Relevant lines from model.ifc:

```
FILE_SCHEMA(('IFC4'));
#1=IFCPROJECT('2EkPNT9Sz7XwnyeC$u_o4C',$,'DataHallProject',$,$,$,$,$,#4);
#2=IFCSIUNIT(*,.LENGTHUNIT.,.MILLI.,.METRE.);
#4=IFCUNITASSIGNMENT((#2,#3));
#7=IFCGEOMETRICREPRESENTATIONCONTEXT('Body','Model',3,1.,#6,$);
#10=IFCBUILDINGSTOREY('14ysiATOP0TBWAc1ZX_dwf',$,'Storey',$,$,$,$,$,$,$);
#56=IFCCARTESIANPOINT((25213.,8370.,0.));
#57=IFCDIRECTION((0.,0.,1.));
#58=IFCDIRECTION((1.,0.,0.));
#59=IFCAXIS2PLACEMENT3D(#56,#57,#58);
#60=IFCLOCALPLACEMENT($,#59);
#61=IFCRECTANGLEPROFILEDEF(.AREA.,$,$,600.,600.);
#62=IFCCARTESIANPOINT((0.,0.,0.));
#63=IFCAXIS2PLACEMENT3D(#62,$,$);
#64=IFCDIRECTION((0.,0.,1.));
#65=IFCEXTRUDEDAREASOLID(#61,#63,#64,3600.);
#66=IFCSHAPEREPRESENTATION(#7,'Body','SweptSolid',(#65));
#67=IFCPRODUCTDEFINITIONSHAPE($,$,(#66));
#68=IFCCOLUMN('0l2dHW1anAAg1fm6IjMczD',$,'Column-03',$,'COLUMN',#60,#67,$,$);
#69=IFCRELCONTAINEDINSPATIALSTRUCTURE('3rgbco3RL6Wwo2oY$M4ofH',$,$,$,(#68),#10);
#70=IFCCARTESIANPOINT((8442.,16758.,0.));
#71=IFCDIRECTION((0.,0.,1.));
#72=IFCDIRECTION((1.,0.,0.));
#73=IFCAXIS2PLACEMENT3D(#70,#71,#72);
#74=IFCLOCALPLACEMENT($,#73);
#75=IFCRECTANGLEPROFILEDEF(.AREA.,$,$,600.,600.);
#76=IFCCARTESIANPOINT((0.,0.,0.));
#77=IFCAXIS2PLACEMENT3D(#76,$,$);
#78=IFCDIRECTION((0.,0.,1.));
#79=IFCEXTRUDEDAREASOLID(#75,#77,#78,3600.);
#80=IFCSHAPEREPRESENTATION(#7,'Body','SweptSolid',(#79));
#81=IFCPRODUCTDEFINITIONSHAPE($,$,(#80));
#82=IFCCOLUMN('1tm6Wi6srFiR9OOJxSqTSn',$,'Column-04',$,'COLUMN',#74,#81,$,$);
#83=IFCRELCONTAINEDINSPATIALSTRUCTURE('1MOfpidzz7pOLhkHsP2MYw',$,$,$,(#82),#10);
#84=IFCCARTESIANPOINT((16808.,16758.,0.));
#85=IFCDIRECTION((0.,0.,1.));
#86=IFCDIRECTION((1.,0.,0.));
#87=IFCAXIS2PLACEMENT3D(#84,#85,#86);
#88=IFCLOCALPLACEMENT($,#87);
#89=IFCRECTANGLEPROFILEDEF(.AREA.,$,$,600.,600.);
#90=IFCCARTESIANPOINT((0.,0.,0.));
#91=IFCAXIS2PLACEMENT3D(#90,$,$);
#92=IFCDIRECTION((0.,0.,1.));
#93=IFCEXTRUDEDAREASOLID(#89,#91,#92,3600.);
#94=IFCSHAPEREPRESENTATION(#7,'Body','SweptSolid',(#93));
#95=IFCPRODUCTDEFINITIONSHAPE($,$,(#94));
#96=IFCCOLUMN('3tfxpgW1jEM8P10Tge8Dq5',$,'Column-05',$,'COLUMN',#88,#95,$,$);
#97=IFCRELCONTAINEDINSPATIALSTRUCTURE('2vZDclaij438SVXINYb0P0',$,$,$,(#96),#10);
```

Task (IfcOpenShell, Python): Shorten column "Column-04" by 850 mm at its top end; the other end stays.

```python
import ifcopenshell
import ifcopenshell.util.unit

model = ifcopenshell.open("model.ifc")
unit_scale = ifcopenshell.util.unit.calculate_unit_scale(model)

member = model.by_guid("1tm6Wi6srFiR9OOJxSqTSn")
change = -0.85 / unit_scale

# The extrusion runs towards the end named, so only its depth changes.
body = next(r for r in member.Representation.Representations if r.RepresentationIdentifier == "Body")
solid = body.Items[0]
old_length = solid.Depth
solid.Depth += change

print(f"length {old_length:g} -> {solid.Depth:g}")

model.write("model-out.ifc")
```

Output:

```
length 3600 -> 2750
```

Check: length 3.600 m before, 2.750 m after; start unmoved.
